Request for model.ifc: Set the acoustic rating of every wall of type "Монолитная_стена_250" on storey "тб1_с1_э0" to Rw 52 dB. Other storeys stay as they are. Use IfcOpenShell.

First a look at what the model holds.

```python
import ifcopenshell
import ifcopenshell.util.element

model = ifcopenshell.open("model.ifc")
print(model.schema)
storey = next(s for s in model.by_type("IfcBuildingStorey") if s.Name == "тб1_с1_э0")
walls = [e for e in ifcopenshell.util.element.get_decomposition(storey) if e.is_a("IfcWall")]
seen = {}
for e in walls:
    element_type = ifcopenshell.util.element.get_type(e)
    key = (element_type.Name if element_type != e and element_type else None, ifcopenshell.util.element.get_pset(e, "Pset_WallCommon", "AcousticRating"))
    seen[key] = seen.get(key, 0) + 1
for (name, value), count in sorted(seen.items(), key=str):
    print(count, "x", name, "|", value)
```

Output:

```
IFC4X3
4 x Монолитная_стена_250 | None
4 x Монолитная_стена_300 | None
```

```python
import ifcopenshell
import ifcopenshell.api.pset
import ifcopenshell.util.element

model = ifcopenshell.open("model.ifc")

storey = next(s for s in model.by_type("IfcBuildingStorey") if s.Name == "тб1_с1_э0")
walls = [e for e in ifcopenshell.util.element.get_decomposition(storey) if e.is_a("IfcWall")]

count = 0
for e in walls:
    element_type = ifcopenshell.util.element.get_type(e)
    if element_type in (None, e) or element_type.Name != "Монолитная_стена_250":
        continue
    # add_pset returns the element's existing set when there is one.
    pset = ifcopenshell.api.pset.add_pset(model, product=e, name="Pset_WallCommon")
    ifcopenshell.api.pset.edit_pset(model, pset=pset, properties={"AcousticRating": "Rw 52 dB"})
    count += 1

print(count, "walls updated")

model.write("model_v2.ifc")
```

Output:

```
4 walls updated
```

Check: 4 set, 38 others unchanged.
